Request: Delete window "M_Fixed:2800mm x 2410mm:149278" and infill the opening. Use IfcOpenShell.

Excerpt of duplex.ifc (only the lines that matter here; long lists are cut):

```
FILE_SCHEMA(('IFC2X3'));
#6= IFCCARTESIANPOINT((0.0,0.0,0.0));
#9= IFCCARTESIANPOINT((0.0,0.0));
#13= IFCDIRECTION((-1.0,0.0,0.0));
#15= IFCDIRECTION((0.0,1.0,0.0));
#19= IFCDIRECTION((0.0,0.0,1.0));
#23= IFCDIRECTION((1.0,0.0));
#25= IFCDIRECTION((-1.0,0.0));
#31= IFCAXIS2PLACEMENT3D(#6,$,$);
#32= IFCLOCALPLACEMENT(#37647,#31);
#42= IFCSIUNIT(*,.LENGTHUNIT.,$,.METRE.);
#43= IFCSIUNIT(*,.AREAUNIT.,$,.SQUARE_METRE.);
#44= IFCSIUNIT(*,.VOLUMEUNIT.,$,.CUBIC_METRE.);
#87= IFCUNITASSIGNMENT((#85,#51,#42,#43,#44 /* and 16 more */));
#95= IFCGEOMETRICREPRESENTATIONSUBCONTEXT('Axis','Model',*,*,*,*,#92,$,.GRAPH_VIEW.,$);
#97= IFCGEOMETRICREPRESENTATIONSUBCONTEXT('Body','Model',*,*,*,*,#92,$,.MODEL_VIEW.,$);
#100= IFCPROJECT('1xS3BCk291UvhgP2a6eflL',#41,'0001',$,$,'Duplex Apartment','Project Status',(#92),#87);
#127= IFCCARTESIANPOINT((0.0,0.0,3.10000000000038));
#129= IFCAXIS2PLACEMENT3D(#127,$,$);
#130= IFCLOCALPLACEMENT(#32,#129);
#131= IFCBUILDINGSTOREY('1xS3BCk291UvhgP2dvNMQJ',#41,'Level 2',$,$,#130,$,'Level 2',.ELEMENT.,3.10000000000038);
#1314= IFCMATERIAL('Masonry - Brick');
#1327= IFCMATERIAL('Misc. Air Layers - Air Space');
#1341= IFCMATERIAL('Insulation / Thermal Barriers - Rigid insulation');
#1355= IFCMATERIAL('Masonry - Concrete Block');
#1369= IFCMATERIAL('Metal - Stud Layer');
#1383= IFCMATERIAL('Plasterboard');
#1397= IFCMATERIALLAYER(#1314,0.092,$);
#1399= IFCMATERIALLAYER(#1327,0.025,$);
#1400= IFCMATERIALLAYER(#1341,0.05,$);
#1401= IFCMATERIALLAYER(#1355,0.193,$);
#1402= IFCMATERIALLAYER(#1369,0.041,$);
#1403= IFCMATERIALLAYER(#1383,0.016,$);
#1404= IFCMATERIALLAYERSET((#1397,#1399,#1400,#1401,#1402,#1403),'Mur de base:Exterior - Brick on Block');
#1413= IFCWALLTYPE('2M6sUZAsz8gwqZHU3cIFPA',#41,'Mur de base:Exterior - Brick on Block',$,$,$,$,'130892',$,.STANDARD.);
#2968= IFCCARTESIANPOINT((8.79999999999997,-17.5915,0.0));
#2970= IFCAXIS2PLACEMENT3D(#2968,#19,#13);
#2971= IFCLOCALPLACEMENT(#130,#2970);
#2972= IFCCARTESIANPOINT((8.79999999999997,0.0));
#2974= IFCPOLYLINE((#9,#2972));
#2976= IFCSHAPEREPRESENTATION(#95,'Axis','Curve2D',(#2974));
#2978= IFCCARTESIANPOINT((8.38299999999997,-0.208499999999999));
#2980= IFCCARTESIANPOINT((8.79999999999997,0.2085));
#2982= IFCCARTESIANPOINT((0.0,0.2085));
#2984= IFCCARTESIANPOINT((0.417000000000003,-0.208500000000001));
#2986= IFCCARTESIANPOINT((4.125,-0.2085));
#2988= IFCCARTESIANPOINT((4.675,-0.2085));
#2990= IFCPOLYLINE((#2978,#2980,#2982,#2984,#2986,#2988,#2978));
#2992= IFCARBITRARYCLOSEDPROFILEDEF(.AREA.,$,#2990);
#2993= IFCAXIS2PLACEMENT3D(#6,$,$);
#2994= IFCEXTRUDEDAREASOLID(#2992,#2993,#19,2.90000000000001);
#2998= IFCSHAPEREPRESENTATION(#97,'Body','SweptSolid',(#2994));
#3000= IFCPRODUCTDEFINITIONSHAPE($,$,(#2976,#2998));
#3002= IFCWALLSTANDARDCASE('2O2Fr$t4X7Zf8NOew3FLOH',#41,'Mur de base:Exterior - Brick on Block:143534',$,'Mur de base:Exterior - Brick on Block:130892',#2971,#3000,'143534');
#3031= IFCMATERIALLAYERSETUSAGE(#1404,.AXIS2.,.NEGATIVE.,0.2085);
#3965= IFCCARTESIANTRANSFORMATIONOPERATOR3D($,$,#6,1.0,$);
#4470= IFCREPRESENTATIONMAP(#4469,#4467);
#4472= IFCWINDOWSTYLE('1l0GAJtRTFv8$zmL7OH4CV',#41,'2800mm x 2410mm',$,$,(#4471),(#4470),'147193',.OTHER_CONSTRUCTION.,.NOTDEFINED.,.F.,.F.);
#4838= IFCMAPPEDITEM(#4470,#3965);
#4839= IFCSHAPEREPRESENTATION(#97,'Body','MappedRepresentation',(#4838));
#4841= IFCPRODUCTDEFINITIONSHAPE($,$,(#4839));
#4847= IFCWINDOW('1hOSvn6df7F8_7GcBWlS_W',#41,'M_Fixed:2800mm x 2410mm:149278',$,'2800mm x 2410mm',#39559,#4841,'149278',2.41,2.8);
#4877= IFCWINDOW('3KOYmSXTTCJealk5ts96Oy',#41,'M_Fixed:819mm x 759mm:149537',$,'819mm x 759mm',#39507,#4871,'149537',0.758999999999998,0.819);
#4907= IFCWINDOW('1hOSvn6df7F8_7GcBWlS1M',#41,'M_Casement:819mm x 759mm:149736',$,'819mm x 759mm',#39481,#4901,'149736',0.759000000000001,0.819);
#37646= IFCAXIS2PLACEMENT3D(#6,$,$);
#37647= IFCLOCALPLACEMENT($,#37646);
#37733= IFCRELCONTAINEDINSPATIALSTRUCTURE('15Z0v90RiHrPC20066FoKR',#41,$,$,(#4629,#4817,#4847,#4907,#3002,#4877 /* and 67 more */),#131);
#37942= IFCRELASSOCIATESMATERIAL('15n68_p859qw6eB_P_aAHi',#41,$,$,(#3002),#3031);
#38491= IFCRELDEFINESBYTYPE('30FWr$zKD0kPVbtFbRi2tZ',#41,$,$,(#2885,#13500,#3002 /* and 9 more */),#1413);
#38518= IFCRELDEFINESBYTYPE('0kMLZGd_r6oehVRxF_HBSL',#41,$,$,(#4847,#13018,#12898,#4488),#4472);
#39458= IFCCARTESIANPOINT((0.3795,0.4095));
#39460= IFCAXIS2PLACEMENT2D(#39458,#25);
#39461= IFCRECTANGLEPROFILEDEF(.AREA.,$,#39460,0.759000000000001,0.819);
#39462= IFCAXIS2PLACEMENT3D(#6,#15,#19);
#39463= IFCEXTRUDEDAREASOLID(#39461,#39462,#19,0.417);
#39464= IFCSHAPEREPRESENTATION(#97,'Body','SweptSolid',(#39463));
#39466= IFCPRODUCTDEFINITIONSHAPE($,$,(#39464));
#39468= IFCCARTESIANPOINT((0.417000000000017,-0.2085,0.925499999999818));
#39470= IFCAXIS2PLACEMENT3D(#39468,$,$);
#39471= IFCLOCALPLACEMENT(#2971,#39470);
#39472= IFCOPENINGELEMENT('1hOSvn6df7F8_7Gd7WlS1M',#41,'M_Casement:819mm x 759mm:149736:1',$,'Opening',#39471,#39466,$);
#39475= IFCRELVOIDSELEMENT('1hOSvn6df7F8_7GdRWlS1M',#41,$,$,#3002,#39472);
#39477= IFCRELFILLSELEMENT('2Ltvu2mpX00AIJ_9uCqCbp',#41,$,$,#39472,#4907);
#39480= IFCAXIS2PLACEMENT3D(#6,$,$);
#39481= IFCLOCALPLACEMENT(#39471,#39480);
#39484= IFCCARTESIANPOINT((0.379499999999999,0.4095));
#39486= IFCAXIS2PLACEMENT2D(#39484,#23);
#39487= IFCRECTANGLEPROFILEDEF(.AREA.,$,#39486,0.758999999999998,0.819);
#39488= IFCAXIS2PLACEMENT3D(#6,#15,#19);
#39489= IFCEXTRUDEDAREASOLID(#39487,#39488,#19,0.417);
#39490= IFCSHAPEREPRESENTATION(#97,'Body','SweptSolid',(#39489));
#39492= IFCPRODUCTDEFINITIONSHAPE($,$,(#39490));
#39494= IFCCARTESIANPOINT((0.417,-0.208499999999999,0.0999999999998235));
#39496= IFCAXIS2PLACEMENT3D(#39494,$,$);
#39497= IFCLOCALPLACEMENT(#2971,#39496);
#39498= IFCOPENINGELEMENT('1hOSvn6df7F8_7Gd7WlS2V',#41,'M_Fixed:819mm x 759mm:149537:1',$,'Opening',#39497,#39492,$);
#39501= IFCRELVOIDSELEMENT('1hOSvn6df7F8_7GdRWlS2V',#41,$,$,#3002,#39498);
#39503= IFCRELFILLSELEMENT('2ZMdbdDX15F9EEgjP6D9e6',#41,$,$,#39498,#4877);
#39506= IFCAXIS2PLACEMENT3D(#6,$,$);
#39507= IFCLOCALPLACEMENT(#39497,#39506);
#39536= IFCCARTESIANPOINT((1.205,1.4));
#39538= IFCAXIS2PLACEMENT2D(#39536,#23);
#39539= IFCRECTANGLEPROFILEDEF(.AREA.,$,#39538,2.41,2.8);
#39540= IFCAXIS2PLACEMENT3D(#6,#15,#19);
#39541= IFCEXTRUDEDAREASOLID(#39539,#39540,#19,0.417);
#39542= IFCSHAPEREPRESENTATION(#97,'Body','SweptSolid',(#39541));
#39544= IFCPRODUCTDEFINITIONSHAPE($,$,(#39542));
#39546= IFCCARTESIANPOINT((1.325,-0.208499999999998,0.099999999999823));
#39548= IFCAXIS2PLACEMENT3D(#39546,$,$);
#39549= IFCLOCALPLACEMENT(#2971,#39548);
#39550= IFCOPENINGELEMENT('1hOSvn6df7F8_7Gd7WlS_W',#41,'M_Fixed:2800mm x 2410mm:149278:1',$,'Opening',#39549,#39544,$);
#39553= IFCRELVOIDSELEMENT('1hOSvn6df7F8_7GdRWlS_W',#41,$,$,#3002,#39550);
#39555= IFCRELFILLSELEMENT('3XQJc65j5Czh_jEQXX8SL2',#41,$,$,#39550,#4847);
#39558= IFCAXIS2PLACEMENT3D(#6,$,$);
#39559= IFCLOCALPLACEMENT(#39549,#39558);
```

```python
import ifcopenshell
import ifcopenshell.api.feature
import ifcopenshell.api.root
import ifcopenshell.geom
import ifcopenshell.util.shape

model = ifcopenshell.open("duplex.ifc")
settings = ifcopenshell.geom.settings()


def volume(element):
    """Net volume in cubic metres, openings subtracted."""
    shape = ifcopenshell.geom.create_shape(settings, element)
    return ifcopenshell.util.shape.get_volume(shape.geometry)


window = model.by_guid("1hOSvn6df7F8_7GcBWlS_W")
opening = window.FillsVoids[0].RelatingOpeningElement
wall = opening.VoidsElements[0].RelatingBuildingElement
before = volume(wall)

ifcopenshell.api.root.remove_product(model, product=window)
ifcopenshell.api.feature.remove_feature(model, feature=opening)

after = volume(wall)

print(f"wall volume {before:.3f} -> {after:.3f} m3")

model.write("duplex_updated.ifc")
```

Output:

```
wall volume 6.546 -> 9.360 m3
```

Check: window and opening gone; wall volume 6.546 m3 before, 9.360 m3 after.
